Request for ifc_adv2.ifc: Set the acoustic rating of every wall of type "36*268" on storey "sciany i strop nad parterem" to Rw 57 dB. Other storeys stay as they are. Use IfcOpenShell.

First a look at what the model holds.

```python
import ifcopenshell
import ifcopenshell.util.element

model = ifcopenshell.open("ifc_adv2.ifc")
print(model.schema)
storey = next(s for s in model.by_type("IfcBuildingStorey") if s.Name == "sciany i strop nad parterem")
walls = [e for e in ifcopenshell.util.element.get_decomposition(storey) if e.is_a("IfcWall")]
seen = {}
for e in walls:
    element_type = ifcopenshell.util.element.get_type(e)
    key = (element_type.Name if element_type != e and element_type else None, ifcopenshell.util.element.get_pset(e, "Pset_WallCommon", "AcousticRating"))
    seen[key] = seen.get(key, 0) + 1
for (name, value), count in sorted(seen.items(), key=str):
    print(count, "x", name, "|", value)
```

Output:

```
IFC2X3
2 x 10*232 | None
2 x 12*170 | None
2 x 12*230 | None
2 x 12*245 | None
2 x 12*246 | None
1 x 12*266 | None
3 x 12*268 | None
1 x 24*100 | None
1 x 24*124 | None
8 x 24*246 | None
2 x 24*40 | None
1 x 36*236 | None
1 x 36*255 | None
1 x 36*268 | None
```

```python
import ifcopenshell
import ifcopenshell.api.pset
import ifcopenshell.util.element

model = ifcopenshell.open("ifc_adv2.ifc")

storey = next(s for s in model.by_type("IfcBuildingStorey") if s.Name == "sciany i strop nad parterem")
walls = [e for e in ifcopenshell.util.element.get_decomposition(storey) if e.is_a("IfcWall")]

count = 0
for e in walls:
    element_type = ifcopenshell.util.element.get_type(e)
    if element_type in (None, e) or element_type.Name != "36*268":
        continue
    # add_pset returns the element's existing set when there is one.
    pset = ifcopenshell.api.pset.add_pset(model, product=e, name="Pset_WallCommon")
    ifcopenshell.api.pset.edit_pset(model, pset=pset, properties={"AcousticRating": "Rw 57 dB"})
    count += 1

print(count, "walls updated")

model.write("ifc_adv2_rev.ifc")
```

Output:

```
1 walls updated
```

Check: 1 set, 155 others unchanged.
